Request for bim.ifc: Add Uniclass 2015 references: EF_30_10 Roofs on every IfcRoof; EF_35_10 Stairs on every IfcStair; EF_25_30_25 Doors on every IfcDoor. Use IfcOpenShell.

First a look at what the model holds.

```python
import ifcopenshell

model = ifcopenshell.open("bim.ifc")
print(model.schema)
print("classifications:", [c.Name for c in model.by_type("IfcClassification")])
for ifc_class in ("IfcDoor", "IfcRoof", "IfcStair", "IfcWall", "IfcWindow"):
    print(ifc_class, len(model.by_type(ifc_class)))
```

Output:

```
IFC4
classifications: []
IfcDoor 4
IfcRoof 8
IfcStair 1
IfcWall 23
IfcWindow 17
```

```python
import ifcopenshell
import ifcopenshell.api.classification

model = ifcopenshell.open("bim.ifc")

system = ifcopenshell.api.classification.add_classification(model, classification="Uniclass 2015")

codes = {
    "IfcRoof": ("EF_30_10", "Roofs"),
    "IfcStair": ("EF_35_10", "Stairs"),
    "IfcDoor": ("EF_25_30_25", "Doors"),
}
for ifc_class, (code, name) in codes.items():
    products = model.by_type(ifc_class)
    ifcopenshell.api.classification.add_reference(
        model, products=products, classification=system, identification=code, name=name
    )
    print(code, len(products))

model.write("bim_updated.ifc")
```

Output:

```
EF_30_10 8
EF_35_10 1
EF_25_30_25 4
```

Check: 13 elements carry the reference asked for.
